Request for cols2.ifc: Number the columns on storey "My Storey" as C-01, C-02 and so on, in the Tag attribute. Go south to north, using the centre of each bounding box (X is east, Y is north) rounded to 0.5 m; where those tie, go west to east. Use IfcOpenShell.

First a look at what the model holds.

```python
import ifcopenshell
import ifcopenshell.util.element
import ifcopenshell.util.placement

model = ifcopenshell.open("cols2.ifc")
print(model.schema)
storey = next(s for s in model.by_type("IfcBuildingStorey") if s.Name == "My Storey")
columns = [e for e in ifcopenshell.util.element.get_decomposition(storey) if e.is_a("IfcColumn")]
for e in sorted(columns, key=lambda e: e.id()):
    origin = ifcopenshell.util.placement.get_local_placement(e.ObjectPlacement)[:3, 3]
    print(e.id(), e.Tag, e.Name, origin.round(2) + 0.0, sep=" | ")
```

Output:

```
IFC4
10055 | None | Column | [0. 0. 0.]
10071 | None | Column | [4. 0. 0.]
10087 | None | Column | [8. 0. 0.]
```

```python
import ifcopenshell
import ifcopenshell.geom
import ifcopenshell.util.element
import ifcopenshell.util.shape

model = ifcopenshell.open("cols2.ifc")
settings = ifcopenshell.geom.settings()
settings.set("use-world-coords", True)


def centre(element):
    shape = ifcopenshell.geom.create_shape(settings, element)
    return ifcopenshell.util.shape.get_bbox_centroid(shape.geometry)


storey = next(s for s in model.by_type("IfcBuildingStorey") if s.Name == "My Storey")
columns = [e for e in ifcopenshell.util.element.get_decomposition(storey) if e.is_a("IfcColumn")]

# Insertion points can sit at a corner or the storey origin, so sort by the geometry (in metres).
centres = {e: centre(e) for e in columns}
columns.sort(key=lambda e: (round(centres[e][1] / 0.5), centres[e][0]))

for i, e in enumerate(columns, start=1):
    number = f"C-{i:02d}"
    e.Tag = number
    print(e.id(), number)

model.write("cols2_edited.ifc")
```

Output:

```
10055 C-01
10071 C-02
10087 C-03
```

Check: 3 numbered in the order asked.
